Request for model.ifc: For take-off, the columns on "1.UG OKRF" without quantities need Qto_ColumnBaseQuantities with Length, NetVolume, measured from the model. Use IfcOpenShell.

First a look at what the model holds.

```python
import ifcopenshell
import ifcopenshell.util.element
import ifcopenshell.util.unit

model = ifcopenshell.open("model.ifc")
print(model.schema)
for unit_type in ("LENGTHUNIT", "AREAUNIT", "VOLUMEUNIT"):
    print(unit_type, ifcopenshell.util.unit.calculate_unit_scale(model, unit_type))
storey = next(s for s in model.by_type("IfcBuildingStorey") if s.Name == "1.UG OKRF")
columns = [e for e in ifcopenshell.util.element.get_decomposition(storey) if e.is_a("IfcColumn")]
for e in sorted(columns, key=lambda e: e.id()):
    print(e.id(), e.is_a(), e.Name, list(ifcopenshell.util.element.get_psets(e, qtos_only=True)), sep=" | ")
```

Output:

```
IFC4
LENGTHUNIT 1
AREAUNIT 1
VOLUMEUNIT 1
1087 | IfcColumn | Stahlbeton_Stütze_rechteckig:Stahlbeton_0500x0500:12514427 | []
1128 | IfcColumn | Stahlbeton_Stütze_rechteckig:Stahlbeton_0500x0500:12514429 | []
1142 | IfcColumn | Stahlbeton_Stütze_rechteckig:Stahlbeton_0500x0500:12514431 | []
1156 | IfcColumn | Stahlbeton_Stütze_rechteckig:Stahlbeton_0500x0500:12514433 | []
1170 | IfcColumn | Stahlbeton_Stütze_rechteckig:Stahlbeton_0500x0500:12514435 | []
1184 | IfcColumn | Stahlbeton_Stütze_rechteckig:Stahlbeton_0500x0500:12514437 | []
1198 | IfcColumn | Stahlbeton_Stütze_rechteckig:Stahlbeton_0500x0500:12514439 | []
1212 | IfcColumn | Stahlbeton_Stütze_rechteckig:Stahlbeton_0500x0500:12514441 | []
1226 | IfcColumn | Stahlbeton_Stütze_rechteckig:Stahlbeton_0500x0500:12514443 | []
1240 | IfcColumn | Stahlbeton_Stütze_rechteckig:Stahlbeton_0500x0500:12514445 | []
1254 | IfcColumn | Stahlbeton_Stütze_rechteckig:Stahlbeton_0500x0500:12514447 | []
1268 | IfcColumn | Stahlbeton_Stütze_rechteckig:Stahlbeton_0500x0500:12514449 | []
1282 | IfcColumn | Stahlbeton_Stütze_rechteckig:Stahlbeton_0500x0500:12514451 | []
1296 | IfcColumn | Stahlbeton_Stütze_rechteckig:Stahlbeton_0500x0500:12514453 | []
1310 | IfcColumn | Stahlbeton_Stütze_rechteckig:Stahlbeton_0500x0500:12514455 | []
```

```python
import ifcopenshell
import ifcopenshell.api.pset
import ifcopenshell.geom
import ifcopenshell.util.element
import ifcopenshell.util.shape
import ifcopenshell.util.unit

model = ifcopenshell.open("model.ifc")
unit_scale = ifcopenshell.util.unit.calculate_unit_scale(model)
volume_scale = ifcopenshell.util.unit.calculate_unit_scale(model, "VOLUMEUNIT")
settings = ifcopenshell.geom.settings()

storey = next(s for s in model.by_type("IfcBuildingStorey") if s.Name == "1.UG OKRF")
columns = [e for e in ifcopenshell.util.element.get_decomposition(storey) if e.is_a("IfcColumn")]

for e in sorted(columns, key=lambda e: e.id()):
    if ifcopenshell.util.element.get_psets(e, qtos_only=True, should_inherit=False):
        continue
    # Geometry comes back in metres, in the element's own axes.
    shape = ifcopenshell.geom.create_shape(settings, e)
    values = {
        "Length": ifcopenshell.util.shape.get_z(shape.geometry) / unit_scale,
        "NetVolume": ifcopenshell.util.shape.get_volume(shape.geometry) / volume_scale,
    }
    qto = ifcopenshell.api.pset.add_qto(model, product=e, name="Qto_ColumnBaseQuantities")
    ifcopenshell.api.pset.edit_qto(model, qto=qto, properties=values)
    print(e.id(), {k: round(v, 3) for k, v in values.items()})

model.write("model_rev.ifc")
```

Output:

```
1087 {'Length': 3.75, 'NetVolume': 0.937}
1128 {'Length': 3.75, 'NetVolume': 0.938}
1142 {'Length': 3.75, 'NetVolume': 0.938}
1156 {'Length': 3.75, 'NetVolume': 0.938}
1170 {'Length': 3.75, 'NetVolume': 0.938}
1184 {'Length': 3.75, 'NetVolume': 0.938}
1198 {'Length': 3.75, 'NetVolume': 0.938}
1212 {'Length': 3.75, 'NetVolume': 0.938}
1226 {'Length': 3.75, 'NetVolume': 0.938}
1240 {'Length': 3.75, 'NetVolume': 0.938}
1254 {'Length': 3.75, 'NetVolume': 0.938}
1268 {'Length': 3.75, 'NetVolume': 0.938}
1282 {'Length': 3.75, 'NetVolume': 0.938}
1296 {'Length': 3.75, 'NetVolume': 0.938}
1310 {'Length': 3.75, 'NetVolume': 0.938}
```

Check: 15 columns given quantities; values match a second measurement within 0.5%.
